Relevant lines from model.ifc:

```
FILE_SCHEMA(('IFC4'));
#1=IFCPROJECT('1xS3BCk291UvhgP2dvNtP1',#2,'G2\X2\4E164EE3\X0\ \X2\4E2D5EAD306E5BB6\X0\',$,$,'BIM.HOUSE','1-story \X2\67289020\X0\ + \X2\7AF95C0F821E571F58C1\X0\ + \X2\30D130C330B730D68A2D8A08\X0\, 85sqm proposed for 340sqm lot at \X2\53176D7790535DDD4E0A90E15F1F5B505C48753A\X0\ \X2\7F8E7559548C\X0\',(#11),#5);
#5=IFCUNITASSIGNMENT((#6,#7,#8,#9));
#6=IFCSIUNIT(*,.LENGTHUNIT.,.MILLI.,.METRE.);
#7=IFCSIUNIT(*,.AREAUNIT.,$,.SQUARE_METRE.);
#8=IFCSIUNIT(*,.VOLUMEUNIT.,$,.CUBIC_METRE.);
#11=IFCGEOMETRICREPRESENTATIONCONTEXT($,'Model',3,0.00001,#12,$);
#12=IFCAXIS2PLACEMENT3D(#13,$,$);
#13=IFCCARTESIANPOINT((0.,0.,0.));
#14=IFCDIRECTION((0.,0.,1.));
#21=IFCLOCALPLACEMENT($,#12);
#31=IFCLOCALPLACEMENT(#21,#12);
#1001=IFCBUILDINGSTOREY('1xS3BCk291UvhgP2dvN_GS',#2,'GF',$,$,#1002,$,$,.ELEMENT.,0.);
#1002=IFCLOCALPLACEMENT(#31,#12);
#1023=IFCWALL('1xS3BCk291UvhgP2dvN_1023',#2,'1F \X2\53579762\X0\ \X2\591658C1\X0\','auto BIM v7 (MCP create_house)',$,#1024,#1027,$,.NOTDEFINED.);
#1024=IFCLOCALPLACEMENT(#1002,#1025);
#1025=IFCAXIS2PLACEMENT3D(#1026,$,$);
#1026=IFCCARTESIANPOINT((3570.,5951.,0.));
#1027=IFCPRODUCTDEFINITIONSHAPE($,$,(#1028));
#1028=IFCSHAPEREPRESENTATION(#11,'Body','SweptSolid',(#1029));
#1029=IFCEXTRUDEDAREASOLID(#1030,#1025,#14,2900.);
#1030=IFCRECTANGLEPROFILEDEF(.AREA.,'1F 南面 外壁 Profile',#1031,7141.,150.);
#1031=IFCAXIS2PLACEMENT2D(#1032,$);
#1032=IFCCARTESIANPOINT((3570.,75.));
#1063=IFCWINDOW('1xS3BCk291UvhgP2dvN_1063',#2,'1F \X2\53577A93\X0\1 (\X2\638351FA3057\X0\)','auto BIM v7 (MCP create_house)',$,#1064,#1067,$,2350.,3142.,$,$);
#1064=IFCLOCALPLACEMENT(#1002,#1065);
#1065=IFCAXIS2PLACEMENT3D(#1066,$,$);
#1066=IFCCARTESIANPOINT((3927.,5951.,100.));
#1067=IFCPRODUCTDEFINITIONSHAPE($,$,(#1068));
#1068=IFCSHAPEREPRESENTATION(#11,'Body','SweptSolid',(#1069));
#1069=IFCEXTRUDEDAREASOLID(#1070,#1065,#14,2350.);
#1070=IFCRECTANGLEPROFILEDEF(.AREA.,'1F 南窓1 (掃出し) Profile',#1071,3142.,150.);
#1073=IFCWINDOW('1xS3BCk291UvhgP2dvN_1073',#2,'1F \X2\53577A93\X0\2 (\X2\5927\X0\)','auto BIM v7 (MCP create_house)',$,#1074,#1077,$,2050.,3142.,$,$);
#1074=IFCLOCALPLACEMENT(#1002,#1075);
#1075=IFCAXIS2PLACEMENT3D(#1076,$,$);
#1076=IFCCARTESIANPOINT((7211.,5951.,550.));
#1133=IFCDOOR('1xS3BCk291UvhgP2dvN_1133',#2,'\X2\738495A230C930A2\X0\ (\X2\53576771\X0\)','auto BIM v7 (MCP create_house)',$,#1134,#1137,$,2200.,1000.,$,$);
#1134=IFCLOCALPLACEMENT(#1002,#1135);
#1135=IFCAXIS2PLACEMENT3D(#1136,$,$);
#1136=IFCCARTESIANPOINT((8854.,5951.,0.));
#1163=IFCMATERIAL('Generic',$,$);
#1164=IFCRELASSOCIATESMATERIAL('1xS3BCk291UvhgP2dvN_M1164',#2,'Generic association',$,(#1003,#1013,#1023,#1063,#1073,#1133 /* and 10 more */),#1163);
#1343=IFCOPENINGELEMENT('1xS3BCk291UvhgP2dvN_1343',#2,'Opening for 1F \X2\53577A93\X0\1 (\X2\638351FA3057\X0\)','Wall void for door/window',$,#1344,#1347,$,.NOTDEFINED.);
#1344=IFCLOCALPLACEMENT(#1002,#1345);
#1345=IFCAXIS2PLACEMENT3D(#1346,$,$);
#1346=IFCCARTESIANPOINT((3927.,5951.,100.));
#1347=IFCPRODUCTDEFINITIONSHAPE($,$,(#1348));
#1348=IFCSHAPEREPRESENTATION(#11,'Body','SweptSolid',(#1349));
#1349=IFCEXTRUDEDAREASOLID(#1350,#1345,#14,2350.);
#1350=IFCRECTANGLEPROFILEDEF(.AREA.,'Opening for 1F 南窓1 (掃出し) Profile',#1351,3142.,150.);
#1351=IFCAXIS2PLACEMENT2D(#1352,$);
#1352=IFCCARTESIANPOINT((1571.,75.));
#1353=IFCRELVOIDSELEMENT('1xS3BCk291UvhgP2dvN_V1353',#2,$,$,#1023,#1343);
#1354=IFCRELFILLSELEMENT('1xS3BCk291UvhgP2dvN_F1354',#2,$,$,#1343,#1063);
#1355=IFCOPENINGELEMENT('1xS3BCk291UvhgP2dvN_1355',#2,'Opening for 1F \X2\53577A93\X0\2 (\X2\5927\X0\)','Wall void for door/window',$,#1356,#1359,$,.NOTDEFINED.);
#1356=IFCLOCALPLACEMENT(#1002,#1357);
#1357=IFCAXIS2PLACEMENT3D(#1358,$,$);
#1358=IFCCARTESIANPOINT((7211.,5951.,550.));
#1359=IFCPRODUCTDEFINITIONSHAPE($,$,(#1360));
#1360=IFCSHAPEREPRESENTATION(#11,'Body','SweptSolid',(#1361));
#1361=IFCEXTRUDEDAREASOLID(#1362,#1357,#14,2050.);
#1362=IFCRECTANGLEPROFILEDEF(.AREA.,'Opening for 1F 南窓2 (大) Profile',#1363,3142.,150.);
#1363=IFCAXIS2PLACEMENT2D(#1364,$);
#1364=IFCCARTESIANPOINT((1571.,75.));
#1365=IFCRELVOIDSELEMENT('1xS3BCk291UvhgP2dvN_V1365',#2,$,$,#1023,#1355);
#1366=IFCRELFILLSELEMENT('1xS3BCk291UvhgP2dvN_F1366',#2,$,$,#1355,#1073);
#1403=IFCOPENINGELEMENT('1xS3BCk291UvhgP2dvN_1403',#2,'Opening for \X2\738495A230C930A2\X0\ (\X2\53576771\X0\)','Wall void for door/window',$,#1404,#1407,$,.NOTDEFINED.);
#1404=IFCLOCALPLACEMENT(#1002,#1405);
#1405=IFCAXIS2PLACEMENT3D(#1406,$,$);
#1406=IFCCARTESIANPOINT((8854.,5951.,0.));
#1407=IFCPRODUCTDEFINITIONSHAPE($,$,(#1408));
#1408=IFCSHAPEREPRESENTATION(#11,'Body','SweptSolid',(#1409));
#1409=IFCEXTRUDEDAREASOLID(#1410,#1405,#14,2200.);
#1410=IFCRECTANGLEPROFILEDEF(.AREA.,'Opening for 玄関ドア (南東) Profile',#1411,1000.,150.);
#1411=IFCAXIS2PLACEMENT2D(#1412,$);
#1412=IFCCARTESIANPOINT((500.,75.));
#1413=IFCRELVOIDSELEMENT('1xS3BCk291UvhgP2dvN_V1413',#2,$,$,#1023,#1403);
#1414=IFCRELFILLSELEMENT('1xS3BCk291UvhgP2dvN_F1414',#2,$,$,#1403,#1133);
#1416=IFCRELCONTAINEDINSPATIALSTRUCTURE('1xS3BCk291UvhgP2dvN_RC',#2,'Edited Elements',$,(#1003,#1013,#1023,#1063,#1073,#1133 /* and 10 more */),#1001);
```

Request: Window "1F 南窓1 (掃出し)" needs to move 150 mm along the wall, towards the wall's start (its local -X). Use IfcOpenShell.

```python
import ifcopenshell
import ifcopenshell.api.geometry
import ifcopenshell.util.placement

model = ifcopenshell.open("model.ifc")

window = model.by_guid("1xS3BCk291UvhgP2dvN_1063")
opening = window.FillsVoids[0].RelatingOpeningElement
wall = opening.VoidsElements[0].RelatingBuildingElement

wall_matrix = ifcopenshell.util.placement.get_local_placement(wall.ObjectPlacement)
shift = wall_matrix[:3, 0] * -150.0
before = ifcopenshell.util.placement.get_local_placement(window.ObjectPlacement)[:3, 3].copy()

# The window is not placed relative to its opening, so move both.
for product in (opening, window):
    matrix = ifcopenshell.util.placement.get_local_placement(product.ObjectPlacement)
    matrix[:3, 3] += shift
    ifcopenshell.api.geometry.edit_object_placement(model, product=product, matrix=matrix, is_si=False)

after = ifcopenshell.util.placement.get_local_placement(window.ObjectPlacement)[:3, 3]
print("window moved by", (after - before).round(3) + 0.0)

model.write("model-out.ifc")
```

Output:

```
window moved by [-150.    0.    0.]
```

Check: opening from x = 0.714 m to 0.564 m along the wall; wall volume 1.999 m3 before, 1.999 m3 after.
